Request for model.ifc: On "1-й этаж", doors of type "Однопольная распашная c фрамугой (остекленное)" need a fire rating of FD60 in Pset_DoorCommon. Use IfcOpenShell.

First a look at what the model holds.

```python
import ifcopenshell
import ifcopenshell.util.element

model = ifcopenshell.open("model.ifc")
print(model.schema)
storey = next(s for s in model.by_type("IfcBuildingStorey") if s.Name == "1-й этаж")
doors = [e for e in ifcopenshell.util.element.get_decomposition(storey) if e.is_a("IfcDoor")]
seen = {}
for e in doors:
    element_type = ifcopenshell.util.element.get_type(e)
    key = (element_type.Name if element_type != e and element_type else None, ifcopenshell.util.element.get_pset(e, "Pset_DoorCommon", "FireRating"))
    seen[key] = seen.get(key, 0) + 1
for (name, value), count in sorted(seen.items(), key=str):
    print(count, "x", name, "|", value)
```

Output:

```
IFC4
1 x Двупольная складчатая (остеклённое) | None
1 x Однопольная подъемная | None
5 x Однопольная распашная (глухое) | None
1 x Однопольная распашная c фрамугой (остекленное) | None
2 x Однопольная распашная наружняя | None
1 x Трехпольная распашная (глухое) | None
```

```python
import ifcopenshell
import ifcopenshell.api.pset
import ifcopenshell.util.element

model = ifcopenshell.open("model.ifc")

storey = next(s for s in model.by_type("IfcBuildingStorey") if s.Name == "1-й этаж")
doors = [e for e in ifcopenshell.util.element.get_decomposition(storey) if e.is_a("IfcDoor")]

count = 0
for e in doors:
    element_type = ifcopenshell.util.element.get_type(e)
    if element_type in (None, e) or element_type.Name != "Однопольная распашная c фрамугой (остекленное)":
        continue
    # add_pset returns the element's existing set when there is one.
    pset = ifcopenshell.api.pset.add_pset(model, product=e, name="Pset_DoorCommon")
    ifcopenshell.api.pset.edit_pset(model, pset=pset, properties={"FireRating": "FD60"})
    count += 1

print(count, "doors updated")

model.write("model-out.ifc")
```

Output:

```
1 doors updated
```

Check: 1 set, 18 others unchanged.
